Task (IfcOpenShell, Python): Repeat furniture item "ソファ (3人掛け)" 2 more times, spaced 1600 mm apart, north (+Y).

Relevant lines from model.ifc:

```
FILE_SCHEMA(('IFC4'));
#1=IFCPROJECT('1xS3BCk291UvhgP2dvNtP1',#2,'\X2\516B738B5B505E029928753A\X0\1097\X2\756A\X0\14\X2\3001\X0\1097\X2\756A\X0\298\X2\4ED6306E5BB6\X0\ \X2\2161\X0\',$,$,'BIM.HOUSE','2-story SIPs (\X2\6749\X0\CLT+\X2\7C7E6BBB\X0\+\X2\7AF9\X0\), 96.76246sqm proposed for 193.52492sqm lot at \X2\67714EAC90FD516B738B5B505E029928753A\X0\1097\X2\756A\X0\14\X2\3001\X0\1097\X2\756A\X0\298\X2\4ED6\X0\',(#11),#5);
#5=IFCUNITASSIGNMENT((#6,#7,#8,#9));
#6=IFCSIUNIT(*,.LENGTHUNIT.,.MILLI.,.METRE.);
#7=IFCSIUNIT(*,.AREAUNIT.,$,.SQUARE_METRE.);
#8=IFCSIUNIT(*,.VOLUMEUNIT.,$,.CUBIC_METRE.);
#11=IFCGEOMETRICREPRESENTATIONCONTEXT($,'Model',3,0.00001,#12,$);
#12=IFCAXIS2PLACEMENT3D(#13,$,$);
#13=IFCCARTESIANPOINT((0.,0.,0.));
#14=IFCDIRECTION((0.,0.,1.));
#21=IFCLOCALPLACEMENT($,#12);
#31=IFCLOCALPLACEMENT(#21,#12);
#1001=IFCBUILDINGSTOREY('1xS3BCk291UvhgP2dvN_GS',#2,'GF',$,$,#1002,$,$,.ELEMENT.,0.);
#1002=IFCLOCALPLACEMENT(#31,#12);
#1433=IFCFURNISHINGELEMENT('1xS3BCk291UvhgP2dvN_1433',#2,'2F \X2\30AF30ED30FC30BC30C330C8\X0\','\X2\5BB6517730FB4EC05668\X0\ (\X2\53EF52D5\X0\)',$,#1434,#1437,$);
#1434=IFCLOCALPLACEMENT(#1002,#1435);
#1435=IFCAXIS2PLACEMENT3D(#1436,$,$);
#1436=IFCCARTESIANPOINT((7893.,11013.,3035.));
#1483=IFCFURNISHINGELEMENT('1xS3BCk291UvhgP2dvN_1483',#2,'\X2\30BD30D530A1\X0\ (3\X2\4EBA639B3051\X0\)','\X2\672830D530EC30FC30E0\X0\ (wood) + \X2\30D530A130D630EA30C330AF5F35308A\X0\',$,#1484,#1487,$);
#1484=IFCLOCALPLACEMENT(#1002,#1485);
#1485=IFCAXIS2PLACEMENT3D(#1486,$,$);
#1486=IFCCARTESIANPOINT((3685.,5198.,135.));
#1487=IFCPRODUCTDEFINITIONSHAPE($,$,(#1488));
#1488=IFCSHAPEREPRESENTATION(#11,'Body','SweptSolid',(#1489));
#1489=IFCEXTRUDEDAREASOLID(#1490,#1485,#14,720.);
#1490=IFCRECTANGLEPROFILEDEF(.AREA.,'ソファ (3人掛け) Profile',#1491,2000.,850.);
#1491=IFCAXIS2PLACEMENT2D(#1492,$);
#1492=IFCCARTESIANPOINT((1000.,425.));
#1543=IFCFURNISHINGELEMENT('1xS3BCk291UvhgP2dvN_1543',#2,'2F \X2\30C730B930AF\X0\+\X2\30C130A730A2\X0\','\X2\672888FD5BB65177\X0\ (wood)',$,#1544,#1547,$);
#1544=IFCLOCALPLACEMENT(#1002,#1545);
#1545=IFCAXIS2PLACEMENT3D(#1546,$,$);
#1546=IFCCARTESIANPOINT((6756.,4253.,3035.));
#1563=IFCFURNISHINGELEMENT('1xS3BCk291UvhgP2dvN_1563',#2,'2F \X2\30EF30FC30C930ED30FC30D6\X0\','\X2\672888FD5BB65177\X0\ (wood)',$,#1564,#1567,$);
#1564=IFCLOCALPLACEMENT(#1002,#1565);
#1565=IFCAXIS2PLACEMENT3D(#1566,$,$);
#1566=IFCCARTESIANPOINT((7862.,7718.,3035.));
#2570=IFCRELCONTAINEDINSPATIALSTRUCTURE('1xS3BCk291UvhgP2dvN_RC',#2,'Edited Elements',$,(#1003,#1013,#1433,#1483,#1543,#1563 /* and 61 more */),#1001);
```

```python
import numpy as np
import ifcopenshell
import ifcopenshell.api.geometry
import ifcopenshell.api.root
import ifcopenshell.util.element
import ifcopenshell.util.placement

model = ifcopenshell.open("model.ifc")


def reuse_history(source, copy):
    """copy_class also copies each property set's owner history, people and application; keep the originals."""
    for rel in copy.IsDefinedBy:
        if rel.is_a("IfcRelDefinesByProperties") and (history := rel.RelatingPropertyDefinition.OwnerHistory):
            rel.RelatingPropertyDefinition.OwnerHistory = source.OwnerHistory
            ifcopenshell.util.element.remove_deep2(model, history)


source = model.by_guid("1xS3BCk291UvhgP2dvN_1483")
base = ifcopenshell.util.placement.get_local_placement(source.ObjectPlacement)
step = np.array([0.0, 1.0, 0.0]) * 1600.0

for i in range(1, 3):
    copy = ifcopenshell.api.root.copy_class(model, product=source)
    copy.Representation = ifcopenshell.util.element.copy_deep(
        model, source.Representation, exclude=["IfcGeometricRepresentationContext", "IfcRepresentationMap"]
    )
    reuse_history(source, copy)
    matrix = base.copy()
    matrix[:3, 3] += i * step
    print("added at", matrix[:3, 3].round(3) + 0.0)
    ifcopenshell.api.geometry.edit_object_placement(model, product=copy, matrix=matrix, is_si=False)

model.write("model-out.ifc")
```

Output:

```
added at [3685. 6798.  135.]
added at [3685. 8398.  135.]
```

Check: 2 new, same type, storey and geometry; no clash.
